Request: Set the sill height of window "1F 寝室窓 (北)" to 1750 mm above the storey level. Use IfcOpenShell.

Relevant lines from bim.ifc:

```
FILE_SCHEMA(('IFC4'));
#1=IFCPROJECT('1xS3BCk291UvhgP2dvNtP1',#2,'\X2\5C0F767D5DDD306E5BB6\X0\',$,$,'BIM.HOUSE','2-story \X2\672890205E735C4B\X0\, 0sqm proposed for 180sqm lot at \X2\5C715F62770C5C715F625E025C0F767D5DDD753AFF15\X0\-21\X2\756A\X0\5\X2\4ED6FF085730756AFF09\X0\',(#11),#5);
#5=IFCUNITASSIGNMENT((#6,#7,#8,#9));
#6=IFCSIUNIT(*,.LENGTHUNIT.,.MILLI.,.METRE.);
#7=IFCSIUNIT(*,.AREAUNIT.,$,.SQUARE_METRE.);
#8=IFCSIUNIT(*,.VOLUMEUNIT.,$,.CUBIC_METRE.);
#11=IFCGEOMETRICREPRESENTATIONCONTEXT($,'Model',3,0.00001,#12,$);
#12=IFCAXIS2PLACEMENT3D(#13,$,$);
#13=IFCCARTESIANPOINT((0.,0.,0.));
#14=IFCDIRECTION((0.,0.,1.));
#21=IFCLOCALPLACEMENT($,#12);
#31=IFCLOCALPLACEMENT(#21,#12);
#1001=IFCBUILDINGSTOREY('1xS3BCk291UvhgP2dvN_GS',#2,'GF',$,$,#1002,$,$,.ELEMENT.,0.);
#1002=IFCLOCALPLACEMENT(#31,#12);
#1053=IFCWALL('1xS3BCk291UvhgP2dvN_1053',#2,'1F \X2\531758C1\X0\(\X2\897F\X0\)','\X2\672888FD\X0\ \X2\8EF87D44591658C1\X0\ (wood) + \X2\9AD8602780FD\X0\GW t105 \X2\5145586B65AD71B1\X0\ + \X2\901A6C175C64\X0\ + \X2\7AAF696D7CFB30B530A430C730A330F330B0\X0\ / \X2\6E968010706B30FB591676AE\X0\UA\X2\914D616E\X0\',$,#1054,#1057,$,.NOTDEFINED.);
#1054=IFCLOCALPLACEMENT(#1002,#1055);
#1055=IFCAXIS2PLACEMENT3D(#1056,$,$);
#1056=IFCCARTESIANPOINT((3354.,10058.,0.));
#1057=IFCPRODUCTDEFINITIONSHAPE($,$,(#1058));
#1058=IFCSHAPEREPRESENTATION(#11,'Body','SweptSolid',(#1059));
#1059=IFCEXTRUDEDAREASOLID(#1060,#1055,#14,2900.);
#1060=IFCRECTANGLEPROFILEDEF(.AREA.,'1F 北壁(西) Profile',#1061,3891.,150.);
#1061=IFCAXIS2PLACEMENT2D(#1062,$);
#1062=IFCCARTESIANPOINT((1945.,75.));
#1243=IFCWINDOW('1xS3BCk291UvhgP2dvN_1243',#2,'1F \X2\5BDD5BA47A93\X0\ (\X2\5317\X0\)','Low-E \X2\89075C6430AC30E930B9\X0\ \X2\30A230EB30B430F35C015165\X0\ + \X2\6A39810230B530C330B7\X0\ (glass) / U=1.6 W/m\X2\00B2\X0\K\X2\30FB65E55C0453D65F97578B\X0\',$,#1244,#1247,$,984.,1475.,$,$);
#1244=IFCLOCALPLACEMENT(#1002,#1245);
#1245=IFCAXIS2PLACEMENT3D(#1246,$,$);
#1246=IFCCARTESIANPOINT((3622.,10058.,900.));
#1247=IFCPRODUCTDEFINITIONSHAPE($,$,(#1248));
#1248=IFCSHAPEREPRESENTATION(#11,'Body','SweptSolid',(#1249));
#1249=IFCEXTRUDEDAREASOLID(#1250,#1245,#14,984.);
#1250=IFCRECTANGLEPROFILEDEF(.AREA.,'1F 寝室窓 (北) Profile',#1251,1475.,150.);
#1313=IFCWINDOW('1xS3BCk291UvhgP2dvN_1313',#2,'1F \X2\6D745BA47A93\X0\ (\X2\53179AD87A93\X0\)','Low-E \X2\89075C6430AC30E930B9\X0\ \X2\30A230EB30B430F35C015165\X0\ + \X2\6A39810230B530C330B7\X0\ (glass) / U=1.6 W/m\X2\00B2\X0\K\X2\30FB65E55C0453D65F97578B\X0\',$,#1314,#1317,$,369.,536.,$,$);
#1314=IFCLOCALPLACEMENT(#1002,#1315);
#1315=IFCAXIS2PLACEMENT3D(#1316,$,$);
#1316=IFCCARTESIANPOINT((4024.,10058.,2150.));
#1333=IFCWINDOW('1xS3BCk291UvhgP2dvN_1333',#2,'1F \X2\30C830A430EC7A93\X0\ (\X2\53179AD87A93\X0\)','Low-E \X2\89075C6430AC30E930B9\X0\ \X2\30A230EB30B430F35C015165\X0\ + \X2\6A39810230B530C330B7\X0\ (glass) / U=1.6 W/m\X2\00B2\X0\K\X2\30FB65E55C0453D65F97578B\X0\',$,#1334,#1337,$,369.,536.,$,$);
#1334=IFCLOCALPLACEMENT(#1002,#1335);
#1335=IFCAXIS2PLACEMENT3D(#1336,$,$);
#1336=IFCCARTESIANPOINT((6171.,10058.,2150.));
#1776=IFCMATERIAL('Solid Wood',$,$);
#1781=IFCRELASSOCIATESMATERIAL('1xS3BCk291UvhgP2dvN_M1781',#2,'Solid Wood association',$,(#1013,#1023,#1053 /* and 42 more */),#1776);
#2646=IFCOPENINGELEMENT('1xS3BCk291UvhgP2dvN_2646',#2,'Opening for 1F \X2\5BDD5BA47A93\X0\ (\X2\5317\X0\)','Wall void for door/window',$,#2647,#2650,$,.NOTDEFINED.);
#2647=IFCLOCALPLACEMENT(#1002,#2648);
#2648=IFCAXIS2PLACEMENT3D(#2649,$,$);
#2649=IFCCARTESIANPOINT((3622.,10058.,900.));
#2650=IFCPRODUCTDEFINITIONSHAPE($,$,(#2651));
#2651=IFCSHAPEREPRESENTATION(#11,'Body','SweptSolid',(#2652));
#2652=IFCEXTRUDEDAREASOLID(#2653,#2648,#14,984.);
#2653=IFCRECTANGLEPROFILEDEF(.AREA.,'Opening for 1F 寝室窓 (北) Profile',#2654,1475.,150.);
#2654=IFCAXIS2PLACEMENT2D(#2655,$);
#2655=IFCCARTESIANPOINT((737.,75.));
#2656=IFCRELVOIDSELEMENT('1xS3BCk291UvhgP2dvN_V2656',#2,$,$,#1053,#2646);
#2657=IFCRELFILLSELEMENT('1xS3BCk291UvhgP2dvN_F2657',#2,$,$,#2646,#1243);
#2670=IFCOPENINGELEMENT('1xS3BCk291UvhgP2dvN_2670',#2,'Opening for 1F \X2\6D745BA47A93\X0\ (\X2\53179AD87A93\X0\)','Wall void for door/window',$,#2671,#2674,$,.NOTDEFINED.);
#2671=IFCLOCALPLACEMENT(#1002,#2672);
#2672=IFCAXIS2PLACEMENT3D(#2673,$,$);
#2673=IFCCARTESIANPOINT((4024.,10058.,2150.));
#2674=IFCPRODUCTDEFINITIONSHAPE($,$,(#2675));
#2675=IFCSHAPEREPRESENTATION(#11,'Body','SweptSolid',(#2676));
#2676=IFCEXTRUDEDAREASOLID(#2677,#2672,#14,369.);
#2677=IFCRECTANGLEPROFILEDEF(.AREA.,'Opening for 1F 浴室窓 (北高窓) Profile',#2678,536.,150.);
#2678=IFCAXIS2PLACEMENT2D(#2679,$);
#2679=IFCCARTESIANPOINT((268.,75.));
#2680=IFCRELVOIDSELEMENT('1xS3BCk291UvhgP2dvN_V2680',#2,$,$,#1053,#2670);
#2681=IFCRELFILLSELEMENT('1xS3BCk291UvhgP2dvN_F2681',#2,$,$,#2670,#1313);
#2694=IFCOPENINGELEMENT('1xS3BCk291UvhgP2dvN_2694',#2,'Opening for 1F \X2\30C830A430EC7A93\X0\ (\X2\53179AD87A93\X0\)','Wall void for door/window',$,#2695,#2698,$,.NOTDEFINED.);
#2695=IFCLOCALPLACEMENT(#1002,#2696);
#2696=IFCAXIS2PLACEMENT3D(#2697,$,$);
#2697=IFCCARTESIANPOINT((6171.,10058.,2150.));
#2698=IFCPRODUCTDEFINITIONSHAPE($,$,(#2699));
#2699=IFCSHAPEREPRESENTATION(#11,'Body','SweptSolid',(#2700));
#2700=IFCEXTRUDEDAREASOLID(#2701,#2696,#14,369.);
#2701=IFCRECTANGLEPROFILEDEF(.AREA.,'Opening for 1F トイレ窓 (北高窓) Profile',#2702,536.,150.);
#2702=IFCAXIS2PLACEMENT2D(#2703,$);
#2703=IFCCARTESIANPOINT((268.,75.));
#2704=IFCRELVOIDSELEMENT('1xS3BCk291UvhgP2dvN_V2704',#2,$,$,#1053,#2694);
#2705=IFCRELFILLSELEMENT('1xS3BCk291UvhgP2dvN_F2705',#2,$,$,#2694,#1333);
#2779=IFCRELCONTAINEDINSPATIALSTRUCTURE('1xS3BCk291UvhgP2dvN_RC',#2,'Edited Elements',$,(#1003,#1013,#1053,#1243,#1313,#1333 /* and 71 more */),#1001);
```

```python
import numpy as np
import ifcopenshell
import ifcopenshell.api.geometry
import ifcopenshell.geom
import ifcopenshell.util.element
import ifcopenshell.util.placement
import ifcopenshell.util.shape
import ifcopenshell.util.unit

model = ifcopenshell.open("bim.ifc")
unit_scale = ifcopenshell.util.unit.calculate_unit_scale(model)

window = model.by_guid("1xS3BCk291UvhgP2dvN_1243")
opening = window.FillsVoids[0].RelatingOpeningElement
storey = ifcopenshell.util.element.get_container(window, ifc_class="IfcBuildingStorey")
level = ifcopenshell.util.placement.get_local_placement(storey.ObjectPlacement)[2, 3]

# The opening's origin need not be at the sill, so measure its lowest point.
shape = ifcopenshell.geom.create_shape(ifcopenshell.geom.settings(), opening)
bottom = ifcopenshell.util.shape.get_shape_bottom_elevation(shape, shape.geometry) / unit_scale
dz = level + 1750.0 - bottom

shift = np.array([0.0, 0.0, dz])
# The window is not placed relative to its opening, so move both.
for product in (opening, window):
    matrix = ifcopenshell.util.placement.get_local_placement(product.ObjectPlacement)
    matrix[:3, 3] += shift
    ifcopenshell.api.geometry.edit_object_placement(model, product=product, matrix=matrix, is_si=False)

print(f"moved by {dz * unit_scale:+.3f} m")

model.write("bim_updated.ifc")
```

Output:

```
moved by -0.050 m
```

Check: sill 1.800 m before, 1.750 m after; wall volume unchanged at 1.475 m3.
